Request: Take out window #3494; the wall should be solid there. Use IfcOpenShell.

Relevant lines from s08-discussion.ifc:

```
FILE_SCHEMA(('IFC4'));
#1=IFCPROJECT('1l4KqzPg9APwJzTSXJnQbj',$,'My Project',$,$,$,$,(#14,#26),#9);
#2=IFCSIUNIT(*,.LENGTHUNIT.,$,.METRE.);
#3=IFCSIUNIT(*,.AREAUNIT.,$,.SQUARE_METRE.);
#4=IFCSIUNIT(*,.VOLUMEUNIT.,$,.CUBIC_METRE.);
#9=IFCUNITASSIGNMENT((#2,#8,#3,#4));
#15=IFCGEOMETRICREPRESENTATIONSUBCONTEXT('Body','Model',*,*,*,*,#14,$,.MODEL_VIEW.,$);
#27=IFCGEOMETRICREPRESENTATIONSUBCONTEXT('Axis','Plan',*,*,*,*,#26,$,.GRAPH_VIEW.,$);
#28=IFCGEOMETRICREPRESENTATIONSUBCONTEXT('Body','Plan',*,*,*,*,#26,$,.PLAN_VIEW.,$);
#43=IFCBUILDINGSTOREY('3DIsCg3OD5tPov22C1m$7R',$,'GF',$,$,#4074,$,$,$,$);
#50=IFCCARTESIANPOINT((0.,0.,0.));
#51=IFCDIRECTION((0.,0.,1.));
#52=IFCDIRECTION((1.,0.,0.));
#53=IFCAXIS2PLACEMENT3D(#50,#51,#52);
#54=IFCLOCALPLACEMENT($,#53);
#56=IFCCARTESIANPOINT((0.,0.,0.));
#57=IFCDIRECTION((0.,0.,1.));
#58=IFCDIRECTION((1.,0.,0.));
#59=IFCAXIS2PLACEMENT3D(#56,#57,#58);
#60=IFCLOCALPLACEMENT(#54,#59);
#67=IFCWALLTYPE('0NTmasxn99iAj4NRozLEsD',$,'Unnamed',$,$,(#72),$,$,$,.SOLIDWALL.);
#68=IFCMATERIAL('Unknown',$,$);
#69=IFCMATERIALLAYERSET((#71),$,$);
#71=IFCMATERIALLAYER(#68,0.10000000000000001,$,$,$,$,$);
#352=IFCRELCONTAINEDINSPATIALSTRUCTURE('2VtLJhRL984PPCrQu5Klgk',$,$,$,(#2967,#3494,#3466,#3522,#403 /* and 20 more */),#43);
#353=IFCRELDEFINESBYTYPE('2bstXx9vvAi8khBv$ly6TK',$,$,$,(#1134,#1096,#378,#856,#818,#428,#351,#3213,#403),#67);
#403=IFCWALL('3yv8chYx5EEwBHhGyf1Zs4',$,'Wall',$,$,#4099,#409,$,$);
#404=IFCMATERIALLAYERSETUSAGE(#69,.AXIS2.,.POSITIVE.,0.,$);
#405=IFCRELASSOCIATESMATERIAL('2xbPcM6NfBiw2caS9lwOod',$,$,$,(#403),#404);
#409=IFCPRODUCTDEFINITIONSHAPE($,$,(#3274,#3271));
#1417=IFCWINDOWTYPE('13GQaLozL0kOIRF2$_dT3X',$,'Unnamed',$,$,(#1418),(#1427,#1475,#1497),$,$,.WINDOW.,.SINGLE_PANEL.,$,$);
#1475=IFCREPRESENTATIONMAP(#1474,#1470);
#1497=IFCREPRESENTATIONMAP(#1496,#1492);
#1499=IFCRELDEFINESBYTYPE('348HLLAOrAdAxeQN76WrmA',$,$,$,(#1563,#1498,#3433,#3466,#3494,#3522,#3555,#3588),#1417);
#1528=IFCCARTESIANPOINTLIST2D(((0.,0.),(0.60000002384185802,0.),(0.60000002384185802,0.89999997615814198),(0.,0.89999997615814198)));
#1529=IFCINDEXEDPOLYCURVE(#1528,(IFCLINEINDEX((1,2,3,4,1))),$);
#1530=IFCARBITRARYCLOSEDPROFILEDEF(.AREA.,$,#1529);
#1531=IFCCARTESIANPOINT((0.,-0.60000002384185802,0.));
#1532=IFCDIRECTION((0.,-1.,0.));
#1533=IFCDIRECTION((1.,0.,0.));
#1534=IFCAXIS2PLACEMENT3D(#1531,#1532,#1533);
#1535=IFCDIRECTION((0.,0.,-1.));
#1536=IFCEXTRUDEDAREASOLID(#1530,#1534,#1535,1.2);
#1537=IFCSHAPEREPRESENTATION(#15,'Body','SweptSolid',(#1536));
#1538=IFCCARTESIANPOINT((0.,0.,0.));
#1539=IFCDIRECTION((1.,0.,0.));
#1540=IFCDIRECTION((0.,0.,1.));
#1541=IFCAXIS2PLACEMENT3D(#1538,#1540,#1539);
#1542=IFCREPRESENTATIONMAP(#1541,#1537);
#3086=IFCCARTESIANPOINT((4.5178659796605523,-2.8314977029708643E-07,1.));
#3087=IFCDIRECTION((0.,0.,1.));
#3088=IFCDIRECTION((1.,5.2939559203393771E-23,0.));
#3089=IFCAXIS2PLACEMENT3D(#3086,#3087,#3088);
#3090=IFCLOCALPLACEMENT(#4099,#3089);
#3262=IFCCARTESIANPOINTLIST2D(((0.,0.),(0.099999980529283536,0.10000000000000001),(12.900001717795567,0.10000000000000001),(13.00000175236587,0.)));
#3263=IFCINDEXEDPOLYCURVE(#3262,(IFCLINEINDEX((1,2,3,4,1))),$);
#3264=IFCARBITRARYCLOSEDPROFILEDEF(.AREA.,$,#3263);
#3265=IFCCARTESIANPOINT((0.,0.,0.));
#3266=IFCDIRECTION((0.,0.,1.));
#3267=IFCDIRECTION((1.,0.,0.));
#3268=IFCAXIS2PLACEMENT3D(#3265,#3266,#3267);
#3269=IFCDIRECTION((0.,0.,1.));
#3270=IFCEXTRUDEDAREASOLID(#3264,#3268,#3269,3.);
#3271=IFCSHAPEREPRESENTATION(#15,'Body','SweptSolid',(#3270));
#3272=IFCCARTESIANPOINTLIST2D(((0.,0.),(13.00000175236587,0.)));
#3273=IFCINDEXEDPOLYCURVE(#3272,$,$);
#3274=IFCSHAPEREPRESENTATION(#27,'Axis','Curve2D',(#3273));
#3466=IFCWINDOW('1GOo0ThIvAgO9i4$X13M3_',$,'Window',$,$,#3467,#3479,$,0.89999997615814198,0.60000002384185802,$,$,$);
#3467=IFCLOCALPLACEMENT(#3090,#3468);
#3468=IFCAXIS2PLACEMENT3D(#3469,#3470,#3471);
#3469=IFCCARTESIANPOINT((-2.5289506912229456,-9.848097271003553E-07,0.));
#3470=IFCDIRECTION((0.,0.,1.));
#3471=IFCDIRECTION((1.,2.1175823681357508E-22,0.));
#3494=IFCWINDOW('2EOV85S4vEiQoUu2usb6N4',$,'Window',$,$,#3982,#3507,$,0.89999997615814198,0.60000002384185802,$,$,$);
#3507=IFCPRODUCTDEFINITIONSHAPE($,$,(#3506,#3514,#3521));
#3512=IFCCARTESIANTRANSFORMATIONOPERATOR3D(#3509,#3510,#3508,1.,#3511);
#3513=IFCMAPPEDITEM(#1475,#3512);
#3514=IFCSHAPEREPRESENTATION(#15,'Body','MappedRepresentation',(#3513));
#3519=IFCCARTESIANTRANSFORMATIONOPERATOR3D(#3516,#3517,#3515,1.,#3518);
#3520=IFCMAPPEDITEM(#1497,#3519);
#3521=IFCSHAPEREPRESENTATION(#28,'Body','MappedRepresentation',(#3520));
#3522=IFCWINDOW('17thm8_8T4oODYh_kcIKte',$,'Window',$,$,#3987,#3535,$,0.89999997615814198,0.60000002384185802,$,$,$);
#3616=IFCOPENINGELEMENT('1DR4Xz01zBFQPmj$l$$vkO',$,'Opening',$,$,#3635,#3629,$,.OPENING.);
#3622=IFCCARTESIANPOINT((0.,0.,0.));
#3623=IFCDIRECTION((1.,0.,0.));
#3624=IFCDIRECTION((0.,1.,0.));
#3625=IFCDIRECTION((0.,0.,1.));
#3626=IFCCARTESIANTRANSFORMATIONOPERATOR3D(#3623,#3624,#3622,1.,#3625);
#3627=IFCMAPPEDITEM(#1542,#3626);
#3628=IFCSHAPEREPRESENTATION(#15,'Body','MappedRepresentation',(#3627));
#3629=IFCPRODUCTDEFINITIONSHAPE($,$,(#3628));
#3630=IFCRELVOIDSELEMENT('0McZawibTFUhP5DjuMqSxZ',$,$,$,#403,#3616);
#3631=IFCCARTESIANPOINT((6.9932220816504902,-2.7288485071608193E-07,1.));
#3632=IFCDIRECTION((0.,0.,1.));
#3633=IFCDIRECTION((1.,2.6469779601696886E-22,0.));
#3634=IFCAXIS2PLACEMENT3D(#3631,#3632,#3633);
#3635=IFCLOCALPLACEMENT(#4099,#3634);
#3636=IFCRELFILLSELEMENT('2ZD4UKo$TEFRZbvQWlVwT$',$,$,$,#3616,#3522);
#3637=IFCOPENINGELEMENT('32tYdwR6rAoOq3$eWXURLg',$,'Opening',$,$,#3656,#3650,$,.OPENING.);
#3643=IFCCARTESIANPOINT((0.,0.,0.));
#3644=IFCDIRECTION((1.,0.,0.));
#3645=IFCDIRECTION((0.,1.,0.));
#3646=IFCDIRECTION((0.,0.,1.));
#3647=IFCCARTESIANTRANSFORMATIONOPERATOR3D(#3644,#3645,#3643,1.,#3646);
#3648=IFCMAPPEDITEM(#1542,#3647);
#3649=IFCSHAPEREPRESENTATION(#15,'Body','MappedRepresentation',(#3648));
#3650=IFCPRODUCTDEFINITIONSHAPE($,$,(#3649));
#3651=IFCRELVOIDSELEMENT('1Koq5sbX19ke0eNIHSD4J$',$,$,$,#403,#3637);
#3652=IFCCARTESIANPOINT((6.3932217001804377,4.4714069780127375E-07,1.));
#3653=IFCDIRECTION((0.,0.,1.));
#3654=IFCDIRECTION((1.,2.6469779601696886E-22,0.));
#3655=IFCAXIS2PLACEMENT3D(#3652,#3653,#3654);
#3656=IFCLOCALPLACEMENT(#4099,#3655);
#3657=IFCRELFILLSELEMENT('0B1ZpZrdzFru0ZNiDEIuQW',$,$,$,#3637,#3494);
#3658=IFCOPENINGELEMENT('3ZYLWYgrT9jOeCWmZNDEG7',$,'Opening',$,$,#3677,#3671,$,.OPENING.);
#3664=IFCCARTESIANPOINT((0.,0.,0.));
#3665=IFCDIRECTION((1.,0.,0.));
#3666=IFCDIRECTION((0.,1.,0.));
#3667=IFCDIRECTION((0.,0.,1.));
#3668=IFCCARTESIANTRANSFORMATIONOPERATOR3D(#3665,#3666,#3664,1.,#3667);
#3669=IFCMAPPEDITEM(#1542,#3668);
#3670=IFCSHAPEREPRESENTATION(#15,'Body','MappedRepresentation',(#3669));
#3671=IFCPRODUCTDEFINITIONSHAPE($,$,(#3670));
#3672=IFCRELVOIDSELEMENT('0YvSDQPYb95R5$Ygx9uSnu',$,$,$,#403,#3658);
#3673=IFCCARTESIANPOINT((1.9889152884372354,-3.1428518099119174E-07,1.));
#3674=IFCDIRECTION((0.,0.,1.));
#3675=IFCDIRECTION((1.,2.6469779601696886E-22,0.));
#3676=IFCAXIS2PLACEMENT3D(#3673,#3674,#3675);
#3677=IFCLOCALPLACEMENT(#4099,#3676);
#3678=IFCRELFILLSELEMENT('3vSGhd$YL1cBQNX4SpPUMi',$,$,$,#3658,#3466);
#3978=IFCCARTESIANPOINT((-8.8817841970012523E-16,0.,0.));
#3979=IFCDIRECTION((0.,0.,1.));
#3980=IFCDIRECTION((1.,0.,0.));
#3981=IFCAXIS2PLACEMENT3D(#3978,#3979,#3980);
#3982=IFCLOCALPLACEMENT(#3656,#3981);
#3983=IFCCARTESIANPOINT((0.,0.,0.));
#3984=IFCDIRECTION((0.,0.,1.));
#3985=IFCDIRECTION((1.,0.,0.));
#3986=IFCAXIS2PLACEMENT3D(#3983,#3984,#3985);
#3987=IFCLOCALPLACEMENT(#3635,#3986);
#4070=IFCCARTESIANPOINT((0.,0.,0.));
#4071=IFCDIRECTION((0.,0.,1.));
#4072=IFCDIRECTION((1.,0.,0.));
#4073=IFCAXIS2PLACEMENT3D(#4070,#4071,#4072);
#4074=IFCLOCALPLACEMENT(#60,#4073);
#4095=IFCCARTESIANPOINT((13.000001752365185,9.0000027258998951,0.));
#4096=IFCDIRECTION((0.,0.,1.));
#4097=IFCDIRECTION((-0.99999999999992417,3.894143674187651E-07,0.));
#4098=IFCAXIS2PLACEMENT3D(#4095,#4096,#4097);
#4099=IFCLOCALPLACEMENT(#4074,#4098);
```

```python
import ifcopenshell
import ifcopenshell.api.feature
import ifcopenshell.api.root
import ifcopenshell.geom
import ifcopenshell.util.shape

model = ifcopenshell.open("s08-discussion.ifc")
settings = ifcopenshell.geom.settings()


def volume(element):
    """Net volume in cubic metres, openings subtracted."""
    shape = ifcopenshell.geom.create_shape(settings, element)
    return ifcopenshell.util.shape.get_volume(shape.geometry)


window = model.by_guid("2EOV85S4vEiQoUu2usb6N4")
opening = window.FillsVoids[0].RelatingOpeningElement
wall = opening.VoidsElements[0].RelatingBuildingElement
before = volume(wall)

ifcopenshell.api.root.remove_product(model, product=window)
ifcopenshell.api.feature.remove_feature(model, feature=opening)

after = volume(wall)

print(f"wall volume {before:.3f} -> {after:.3f} m3")

model.write("s08-discussion_edited.ifc")
```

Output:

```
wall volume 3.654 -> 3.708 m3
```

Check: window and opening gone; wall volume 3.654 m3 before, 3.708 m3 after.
